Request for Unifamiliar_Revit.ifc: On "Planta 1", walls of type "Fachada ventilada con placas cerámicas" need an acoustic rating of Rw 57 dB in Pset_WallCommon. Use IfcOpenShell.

First a look at what the model holds.

```python
import ifcopenshell
import ifcopenshell.util.element

model = ifcopenshell.open("Unifamiliar_Revit.ifc")
print(model.schema)
storey = next(s for s in model.by_type("IfcBuildingStorey") if s.Name == "Planta 1")
walls = [e for e in ifcopenshell.util.element.get_decomposition(storey) if e.is_a("IfcWall")]
seen = {}
for e in walls:
    element_type = ifcopenshell.util.element.get_type(e)
    key = (element_type.Name if element_type != e and element_type else None, ifcopenshell.util.element.get_pset(e, "Pset_WallCommon", "AcousticRating"))
    seen[key] = seen.get(key, 0) + 1
for (name, value), count in sorted(seen.items(), key=str):
    print(count, "x", name, "|", value)
```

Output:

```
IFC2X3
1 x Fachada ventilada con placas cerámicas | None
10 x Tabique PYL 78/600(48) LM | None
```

```python
import ifcopenshell
import ifcopenshell.api.pset
import ifcopenshell.util.element

model = ifcopenshell.open("Unifamiliar_Revit.ifc")

storey = next(s for s in model.by_type("IfcBuildingStorey") if s.Name == "Planta 1")
walls = [e for e in ifcopenshell.util.element.get_decomposition(storey) if e.is_a("IfcWall")]

count = 0
for e in walls:
    element_type = ifcopenshell.util.element.get_type(e)
    if element_type in (None, e) or element_type.Name != "Fachada ventilada con placas cerámicas":
        continue
    # add_pset returns the element's existing set when there is one.
    pset = ifcopenshell.api.pset.add_pset(model, product=e, name="Pset_WallCommon")
    ifcopenshell.api.pset.edit_pset(model, pset=pset, properties={"AcousticRating": "Rw 57 dB"})
    count += 1

print(count, "walls updated")

model.write("Unifamiliar_Revit_rev.ifc")
```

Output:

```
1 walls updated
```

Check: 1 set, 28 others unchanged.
